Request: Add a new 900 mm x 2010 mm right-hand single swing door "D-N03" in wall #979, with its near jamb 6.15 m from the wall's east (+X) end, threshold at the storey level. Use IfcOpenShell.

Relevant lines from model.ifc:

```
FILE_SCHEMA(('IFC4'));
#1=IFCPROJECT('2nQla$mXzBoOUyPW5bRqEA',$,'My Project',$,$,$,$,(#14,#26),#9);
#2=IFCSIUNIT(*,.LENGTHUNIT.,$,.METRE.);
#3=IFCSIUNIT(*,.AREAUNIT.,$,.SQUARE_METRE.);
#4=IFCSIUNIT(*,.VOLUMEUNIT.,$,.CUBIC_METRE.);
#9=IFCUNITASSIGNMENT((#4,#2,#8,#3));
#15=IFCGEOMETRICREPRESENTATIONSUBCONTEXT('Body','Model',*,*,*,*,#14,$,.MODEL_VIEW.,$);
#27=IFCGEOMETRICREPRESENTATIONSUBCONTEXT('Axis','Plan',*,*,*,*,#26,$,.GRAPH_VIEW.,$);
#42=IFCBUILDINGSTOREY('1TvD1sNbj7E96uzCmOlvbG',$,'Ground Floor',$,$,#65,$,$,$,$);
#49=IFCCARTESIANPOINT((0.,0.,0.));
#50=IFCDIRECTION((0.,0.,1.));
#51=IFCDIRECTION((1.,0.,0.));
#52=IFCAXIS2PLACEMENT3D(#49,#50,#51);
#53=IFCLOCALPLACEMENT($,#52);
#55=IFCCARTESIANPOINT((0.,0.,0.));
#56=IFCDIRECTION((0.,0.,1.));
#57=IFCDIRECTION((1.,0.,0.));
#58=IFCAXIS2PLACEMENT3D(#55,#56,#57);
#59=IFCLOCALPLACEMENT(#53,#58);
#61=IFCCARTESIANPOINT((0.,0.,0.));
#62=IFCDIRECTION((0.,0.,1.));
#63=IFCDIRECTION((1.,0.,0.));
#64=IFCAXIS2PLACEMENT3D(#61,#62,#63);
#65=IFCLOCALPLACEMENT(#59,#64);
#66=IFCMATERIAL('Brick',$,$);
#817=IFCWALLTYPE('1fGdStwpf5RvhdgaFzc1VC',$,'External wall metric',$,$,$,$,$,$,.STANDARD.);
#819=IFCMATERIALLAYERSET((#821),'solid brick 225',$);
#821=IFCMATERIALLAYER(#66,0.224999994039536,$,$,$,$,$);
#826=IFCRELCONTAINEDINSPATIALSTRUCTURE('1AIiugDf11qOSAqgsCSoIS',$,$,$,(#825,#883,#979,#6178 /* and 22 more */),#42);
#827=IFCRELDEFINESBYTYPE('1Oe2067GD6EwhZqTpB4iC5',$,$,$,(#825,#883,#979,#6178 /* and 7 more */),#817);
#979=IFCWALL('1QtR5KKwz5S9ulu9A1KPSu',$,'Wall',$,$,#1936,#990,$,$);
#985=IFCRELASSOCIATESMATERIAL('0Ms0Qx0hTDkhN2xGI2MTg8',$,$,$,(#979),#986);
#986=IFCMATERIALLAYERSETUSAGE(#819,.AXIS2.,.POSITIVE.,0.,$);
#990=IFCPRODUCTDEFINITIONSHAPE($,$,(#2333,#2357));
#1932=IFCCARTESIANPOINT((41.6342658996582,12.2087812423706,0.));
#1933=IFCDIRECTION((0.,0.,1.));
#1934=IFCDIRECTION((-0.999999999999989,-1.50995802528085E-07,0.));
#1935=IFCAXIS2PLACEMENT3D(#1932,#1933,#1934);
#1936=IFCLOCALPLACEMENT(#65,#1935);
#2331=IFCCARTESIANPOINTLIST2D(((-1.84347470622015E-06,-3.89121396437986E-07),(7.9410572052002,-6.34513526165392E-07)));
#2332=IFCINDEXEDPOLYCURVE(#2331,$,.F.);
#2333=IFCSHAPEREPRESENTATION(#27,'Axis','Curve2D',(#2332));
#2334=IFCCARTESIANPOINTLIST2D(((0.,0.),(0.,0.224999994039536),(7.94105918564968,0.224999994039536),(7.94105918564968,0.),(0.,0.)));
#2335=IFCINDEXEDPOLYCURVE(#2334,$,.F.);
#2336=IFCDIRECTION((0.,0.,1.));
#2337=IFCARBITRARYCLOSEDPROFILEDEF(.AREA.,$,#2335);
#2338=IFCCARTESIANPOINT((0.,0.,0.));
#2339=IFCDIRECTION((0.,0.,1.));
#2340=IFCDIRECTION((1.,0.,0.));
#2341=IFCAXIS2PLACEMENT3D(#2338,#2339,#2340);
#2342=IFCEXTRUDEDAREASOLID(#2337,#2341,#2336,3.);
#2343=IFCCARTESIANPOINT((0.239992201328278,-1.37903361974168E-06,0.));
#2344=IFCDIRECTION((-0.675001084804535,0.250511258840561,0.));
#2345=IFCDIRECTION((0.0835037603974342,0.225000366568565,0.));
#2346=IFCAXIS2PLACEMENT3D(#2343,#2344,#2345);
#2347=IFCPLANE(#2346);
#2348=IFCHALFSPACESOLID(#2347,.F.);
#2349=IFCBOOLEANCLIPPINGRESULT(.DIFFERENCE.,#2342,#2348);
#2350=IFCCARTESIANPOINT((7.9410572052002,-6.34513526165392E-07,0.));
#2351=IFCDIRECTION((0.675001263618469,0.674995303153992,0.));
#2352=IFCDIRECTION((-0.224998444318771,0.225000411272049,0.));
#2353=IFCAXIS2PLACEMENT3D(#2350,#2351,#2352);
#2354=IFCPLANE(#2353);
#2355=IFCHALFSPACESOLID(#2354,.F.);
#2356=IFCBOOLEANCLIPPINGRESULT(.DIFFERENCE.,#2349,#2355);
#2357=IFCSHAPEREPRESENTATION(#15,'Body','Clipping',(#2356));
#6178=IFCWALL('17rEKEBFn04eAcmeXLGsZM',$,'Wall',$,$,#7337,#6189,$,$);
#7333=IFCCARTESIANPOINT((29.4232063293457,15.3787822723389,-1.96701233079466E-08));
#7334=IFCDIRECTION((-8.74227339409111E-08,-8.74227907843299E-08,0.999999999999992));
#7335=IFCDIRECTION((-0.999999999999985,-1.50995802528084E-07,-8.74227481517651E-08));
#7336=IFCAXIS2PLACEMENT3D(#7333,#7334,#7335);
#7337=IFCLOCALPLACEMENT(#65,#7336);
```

```python
import numpy as np
import ifcopenshell
import ifcopenshell.api.feature
import ifcopenshell.api.geometry
import ifcopenshell.api.root
import ifcopenshell.api.spatial
import ifcopenshell.geom
import ifcopenshell.util.element
import ifcopenshell.util.placement
import ifcopenshell.util.representation
import ifcopenshell.util.shape
import ifcopenshell.util.unit

model = ifcopenshell.open("model.ifc")
unit_scale = ifcopenshell.util.unit.calculate_unit_scale(model)
settings = ifcopenshell.geom.settings()


def volume(element):
    """Net volume in cubic metres, openings subtracted."""
    shape = ifcopenshell.geom.create_shape(settings, element)
    return ifcopenshell.util.shape.get_volume(shape.geometry)


wall = model.by_guid("1QtR5KKwz5S9ulu9A1KPSu")
storey = ifcopenshell.util.element.get_container(wall, ifc_class="IfcBuildingStorey")
context = ifcopenshell.util.representation.get_context(model, "Model", "Body", "MODEL_VIEW")
before = volume(wall)

width, height, from_end, sill = 0.9, 2.01, 6.15, 0.0  # metres

# The wall runs along its own X axis, and the end named is its -X end.
wall_shape = ifcopenshell.geom.create_shape(settings, wall)
x, y, z = ifcopenshell.util.shape.get_vertices(wall_shape.geometry).T
start = x.min() + from_end
face, thickness = float(y.min()), float(y.max() - y.min())
wall_matrix = ifcopenshell.util.placement.get_local_placement(wall.ObjectPlacement)
level = ifcopenshell.util.placement.get_local_placement(storey.ObjectPlacement)[2, 3]


def in_wall(x, y):
    """Placement at x, y metres in the wall's axes, at sill height."""
    matrix = wall_matrix.copy()
    matrix[:, 3] = wall_matrix @ np.array([x / unit_scale, y / unit_scale, 0.0, 1.0])
    matrix[2, 3] = level + sill / unit_scale
    return matrix


# Opening: a box that overshoots both wall faces by 50 mm.
opening = ifcopenshell.api.root.create_entity(model, ifc_class="IfcOpeningElement", predefined_type="OPENING")
box = ifcopenshell.api.geometry.add_wall_representation(
    model, context=context, length=width, height=height, thickness=thickness + 0.1
)
ifcopenshell.api.geometry.assign_representation(model, product=opening, representation=box)
ifcopenshell.api.geometry.edit_object_placement(model, product=opening, matrix=in_wall(start, face - 0.05), is_si=False)
ifcopenshell.api.feature.add_feature(model, feature=opening, element=wall)

door = ifcopenshell.api.root.create_entity(model, ifc_class="IfcDoor", name="D-N03", predefined_type="DOOR")
door.OverallWidth, door.OverallHeight = width / unit_scale, height / unit_scale
door.OperationType = "SINGLE_SWING_RIGHT"
body = ifcopenshell.api.geometry.add_door_representation(
    model,
    context=context,
    overall_width=door.OverallWidth,
    overall_height=door.OverallHeight,
    operation_type="SINGLE_SWING_RIGHT",
    lining_properties={"LiningDepth": thickness / unit_scale, "ThresholdDepth": thickness / unit_scale},
)
ifcopenshell.api.geometry.assign_representation(model, product=door, representation=body)
ifcopenshell.api.spatial.assign_container(model, products=[door], relating_structure=storey)
ifcopenshell.api.feature.add_filling(model, opening=opening, element=door)

# The lining spans the wall, so the door starts at the wall face.
ifcopenshell.api.geometry.edit_object_placement(model, product=door, matrix=in_wall(start, face), is_si=False)

after = volume(wall)

print(f"wall volume {before:.3f} -> {after:.3f} m3")

model.write("model_edited.ifc")
```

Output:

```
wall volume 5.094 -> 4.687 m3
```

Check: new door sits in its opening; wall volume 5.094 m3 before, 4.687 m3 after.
